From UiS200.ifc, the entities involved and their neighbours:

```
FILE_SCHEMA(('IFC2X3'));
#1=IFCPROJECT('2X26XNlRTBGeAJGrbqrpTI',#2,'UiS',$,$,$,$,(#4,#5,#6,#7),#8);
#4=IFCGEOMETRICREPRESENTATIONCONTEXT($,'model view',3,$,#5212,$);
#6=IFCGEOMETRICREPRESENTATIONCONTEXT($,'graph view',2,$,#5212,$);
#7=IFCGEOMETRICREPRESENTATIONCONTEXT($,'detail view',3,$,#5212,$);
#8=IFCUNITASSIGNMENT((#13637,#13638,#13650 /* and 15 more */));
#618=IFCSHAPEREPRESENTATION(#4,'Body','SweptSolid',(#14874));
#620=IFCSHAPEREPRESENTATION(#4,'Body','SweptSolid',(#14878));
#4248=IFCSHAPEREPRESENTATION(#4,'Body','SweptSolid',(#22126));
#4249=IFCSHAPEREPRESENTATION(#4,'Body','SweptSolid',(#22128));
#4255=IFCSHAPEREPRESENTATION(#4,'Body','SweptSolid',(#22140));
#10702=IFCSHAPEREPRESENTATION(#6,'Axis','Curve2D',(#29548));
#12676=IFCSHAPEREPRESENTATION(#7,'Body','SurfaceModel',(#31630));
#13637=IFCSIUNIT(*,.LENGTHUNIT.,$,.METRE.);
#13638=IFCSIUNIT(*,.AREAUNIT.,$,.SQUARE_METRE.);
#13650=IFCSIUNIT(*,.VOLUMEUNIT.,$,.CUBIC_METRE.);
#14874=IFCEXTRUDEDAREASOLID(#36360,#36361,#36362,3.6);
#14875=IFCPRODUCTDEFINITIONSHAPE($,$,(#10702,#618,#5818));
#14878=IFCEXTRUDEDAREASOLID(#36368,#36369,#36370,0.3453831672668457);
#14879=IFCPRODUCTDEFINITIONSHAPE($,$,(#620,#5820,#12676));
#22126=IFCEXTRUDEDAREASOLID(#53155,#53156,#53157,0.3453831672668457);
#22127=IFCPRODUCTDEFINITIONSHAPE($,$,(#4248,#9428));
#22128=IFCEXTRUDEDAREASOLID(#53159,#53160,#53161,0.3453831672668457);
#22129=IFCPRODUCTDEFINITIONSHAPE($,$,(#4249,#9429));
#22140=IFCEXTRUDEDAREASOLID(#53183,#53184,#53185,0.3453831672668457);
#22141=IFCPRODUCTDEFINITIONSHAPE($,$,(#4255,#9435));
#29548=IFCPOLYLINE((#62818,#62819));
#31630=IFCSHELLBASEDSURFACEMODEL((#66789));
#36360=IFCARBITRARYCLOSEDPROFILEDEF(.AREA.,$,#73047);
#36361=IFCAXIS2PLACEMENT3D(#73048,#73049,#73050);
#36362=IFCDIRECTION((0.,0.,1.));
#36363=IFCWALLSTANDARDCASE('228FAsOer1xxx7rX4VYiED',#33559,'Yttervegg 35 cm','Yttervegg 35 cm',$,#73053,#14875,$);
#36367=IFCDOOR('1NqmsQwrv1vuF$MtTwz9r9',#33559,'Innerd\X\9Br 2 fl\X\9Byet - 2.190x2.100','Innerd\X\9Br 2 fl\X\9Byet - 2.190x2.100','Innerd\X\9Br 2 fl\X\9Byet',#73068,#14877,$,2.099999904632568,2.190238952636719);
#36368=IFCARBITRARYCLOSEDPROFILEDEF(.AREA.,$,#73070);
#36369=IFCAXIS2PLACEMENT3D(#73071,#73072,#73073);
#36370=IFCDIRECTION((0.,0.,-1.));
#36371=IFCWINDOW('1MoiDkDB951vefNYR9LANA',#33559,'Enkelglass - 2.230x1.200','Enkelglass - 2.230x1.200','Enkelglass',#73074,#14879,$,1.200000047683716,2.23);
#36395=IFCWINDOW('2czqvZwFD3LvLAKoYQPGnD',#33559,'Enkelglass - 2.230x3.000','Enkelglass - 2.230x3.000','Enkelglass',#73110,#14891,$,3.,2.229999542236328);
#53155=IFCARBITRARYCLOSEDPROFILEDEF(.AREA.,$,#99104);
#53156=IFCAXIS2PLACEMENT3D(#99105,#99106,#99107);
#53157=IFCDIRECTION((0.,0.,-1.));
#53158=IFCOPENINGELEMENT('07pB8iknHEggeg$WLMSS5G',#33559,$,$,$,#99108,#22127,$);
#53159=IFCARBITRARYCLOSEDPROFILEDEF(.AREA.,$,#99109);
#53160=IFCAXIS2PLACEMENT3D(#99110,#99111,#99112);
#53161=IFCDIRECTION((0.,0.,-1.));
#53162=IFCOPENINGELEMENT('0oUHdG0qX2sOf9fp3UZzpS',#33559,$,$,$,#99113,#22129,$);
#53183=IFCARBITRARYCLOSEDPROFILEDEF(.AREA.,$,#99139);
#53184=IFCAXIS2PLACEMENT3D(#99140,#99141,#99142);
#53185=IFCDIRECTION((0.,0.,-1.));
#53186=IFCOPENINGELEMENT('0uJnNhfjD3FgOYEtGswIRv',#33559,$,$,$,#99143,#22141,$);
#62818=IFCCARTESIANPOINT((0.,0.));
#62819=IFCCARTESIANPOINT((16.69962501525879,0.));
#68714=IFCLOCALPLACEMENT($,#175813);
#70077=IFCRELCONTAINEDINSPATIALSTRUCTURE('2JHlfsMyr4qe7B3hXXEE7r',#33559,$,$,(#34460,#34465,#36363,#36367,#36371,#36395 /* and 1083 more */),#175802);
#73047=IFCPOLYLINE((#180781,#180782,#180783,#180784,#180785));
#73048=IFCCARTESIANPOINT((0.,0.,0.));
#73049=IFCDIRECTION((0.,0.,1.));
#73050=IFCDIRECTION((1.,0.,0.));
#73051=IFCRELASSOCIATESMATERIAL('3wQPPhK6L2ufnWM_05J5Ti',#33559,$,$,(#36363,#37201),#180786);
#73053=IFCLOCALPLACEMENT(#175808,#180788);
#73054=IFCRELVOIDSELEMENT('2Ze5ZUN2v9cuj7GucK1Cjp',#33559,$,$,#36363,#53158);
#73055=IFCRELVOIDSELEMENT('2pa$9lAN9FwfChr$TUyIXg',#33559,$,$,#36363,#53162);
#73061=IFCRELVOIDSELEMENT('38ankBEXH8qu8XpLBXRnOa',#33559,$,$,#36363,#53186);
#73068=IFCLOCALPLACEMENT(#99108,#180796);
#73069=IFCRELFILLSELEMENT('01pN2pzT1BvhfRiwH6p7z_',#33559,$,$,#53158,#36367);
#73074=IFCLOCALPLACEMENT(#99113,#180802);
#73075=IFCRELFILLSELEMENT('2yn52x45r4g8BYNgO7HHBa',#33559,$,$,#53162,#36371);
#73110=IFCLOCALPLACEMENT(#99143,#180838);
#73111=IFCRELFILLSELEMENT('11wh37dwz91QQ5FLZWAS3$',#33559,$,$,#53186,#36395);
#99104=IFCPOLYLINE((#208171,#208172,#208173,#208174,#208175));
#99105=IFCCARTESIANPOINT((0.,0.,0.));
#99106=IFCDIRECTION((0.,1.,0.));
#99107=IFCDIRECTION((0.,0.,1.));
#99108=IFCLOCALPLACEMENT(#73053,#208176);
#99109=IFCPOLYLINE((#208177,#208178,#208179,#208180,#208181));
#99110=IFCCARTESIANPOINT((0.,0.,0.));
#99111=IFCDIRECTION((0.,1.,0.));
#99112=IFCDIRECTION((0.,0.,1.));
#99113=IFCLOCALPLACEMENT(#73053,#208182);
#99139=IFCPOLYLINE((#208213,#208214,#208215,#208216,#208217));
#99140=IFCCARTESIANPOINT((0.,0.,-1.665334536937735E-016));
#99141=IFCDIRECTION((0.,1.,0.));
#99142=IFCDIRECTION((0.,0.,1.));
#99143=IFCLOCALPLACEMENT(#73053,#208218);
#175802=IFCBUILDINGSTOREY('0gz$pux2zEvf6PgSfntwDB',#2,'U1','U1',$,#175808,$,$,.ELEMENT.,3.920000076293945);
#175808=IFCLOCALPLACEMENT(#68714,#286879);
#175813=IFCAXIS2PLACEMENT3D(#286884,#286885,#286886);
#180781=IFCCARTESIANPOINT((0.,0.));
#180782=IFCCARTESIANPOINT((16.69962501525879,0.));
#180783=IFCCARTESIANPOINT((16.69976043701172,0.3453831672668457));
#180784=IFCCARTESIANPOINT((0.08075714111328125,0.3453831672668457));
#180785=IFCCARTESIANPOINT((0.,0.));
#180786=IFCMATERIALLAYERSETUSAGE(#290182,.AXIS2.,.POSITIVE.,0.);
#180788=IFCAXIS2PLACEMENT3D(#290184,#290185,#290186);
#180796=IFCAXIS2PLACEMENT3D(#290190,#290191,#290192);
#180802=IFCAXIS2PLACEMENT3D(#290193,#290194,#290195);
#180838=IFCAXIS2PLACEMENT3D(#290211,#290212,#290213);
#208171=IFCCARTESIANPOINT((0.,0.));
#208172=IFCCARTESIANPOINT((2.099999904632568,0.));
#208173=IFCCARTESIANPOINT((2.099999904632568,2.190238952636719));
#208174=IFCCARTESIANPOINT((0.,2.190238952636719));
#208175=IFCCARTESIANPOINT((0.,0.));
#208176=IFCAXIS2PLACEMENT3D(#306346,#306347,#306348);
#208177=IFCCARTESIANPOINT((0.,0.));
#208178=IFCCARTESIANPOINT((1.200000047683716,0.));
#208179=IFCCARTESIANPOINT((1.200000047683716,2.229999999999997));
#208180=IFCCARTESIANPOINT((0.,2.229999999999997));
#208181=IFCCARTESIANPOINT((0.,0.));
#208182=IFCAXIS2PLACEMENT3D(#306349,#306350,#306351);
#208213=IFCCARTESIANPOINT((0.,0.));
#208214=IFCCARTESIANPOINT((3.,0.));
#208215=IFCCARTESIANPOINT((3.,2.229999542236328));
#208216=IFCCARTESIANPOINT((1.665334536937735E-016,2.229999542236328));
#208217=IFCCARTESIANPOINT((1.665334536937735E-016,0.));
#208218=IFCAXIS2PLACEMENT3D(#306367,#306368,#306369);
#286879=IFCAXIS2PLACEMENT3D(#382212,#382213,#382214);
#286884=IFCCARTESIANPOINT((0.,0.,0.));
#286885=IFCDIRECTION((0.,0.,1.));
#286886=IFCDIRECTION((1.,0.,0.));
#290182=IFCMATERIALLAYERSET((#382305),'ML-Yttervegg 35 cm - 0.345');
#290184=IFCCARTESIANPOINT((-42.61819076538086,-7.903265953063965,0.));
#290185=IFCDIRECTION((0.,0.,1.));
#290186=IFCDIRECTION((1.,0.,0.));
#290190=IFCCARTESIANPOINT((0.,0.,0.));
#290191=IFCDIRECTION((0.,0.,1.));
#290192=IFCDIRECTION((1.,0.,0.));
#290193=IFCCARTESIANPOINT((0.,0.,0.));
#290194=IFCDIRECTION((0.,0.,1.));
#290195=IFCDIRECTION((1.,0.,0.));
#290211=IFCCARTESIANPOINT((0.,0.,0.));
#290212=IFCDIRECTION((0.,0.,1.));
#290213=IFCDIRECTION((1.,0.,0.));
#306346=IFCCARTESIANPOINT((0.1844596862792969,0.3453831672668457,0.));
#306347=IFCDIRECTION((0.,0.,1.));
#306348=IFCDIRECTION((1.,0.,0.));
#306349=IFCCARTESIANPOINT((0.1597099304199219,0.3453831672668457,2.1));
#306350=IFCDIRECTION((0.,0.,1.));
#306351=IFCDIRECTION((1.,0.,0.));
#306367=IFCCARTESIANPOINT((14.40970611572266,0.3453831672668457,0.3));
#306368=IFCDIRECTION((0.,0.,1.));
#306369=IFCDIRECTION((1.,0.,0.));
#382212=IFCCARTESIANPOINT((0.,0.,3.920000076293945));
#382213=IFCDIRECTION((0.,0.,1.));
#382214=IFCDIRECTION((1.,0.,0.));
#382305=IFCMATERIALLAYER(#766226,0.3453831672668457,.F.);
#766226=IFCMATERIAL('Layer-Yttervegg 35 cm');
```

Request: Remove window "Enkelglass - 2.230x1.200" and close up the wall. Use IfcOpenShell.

```python
import ifcopenshell
import ifcopenshell.api.feature
import ifcopenshell.api.root
import ifcopenshell.geom
import ifcopenshell.util.shape

model = ifcopenshell.open("UiS200.ifc")
settings = ifcopenshell.geom.settings()


def volume(element):
    """Net volume in cubic metres, openings subtracted."""
    shape = ifcopenshell.geom.create_shape(settings, element)
    return ifcopenshell.util.shape.get_volume(shape.geometry)


window = model.by_guid("1MoiDkDB951vefNYR9LANA")
opening = window.FillsVoids[0].RelatingOpeningElement
wall = opening.VoidsElements[0].RelatingBuildingElement
before = volume(wall)

ifcopenshell.api.root.remove_product(model, product=window)
ifcopenshell.api.feature.remove_feature(model, feature=opening)

after = volume(wall)

print(f"wall volume {before:.3f} -> {after:.3f} m3")

model.write("UiS200_updated.ifc")
```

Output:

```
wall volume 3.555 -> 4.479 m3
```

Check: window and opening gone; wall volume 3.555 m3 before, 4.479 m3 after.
